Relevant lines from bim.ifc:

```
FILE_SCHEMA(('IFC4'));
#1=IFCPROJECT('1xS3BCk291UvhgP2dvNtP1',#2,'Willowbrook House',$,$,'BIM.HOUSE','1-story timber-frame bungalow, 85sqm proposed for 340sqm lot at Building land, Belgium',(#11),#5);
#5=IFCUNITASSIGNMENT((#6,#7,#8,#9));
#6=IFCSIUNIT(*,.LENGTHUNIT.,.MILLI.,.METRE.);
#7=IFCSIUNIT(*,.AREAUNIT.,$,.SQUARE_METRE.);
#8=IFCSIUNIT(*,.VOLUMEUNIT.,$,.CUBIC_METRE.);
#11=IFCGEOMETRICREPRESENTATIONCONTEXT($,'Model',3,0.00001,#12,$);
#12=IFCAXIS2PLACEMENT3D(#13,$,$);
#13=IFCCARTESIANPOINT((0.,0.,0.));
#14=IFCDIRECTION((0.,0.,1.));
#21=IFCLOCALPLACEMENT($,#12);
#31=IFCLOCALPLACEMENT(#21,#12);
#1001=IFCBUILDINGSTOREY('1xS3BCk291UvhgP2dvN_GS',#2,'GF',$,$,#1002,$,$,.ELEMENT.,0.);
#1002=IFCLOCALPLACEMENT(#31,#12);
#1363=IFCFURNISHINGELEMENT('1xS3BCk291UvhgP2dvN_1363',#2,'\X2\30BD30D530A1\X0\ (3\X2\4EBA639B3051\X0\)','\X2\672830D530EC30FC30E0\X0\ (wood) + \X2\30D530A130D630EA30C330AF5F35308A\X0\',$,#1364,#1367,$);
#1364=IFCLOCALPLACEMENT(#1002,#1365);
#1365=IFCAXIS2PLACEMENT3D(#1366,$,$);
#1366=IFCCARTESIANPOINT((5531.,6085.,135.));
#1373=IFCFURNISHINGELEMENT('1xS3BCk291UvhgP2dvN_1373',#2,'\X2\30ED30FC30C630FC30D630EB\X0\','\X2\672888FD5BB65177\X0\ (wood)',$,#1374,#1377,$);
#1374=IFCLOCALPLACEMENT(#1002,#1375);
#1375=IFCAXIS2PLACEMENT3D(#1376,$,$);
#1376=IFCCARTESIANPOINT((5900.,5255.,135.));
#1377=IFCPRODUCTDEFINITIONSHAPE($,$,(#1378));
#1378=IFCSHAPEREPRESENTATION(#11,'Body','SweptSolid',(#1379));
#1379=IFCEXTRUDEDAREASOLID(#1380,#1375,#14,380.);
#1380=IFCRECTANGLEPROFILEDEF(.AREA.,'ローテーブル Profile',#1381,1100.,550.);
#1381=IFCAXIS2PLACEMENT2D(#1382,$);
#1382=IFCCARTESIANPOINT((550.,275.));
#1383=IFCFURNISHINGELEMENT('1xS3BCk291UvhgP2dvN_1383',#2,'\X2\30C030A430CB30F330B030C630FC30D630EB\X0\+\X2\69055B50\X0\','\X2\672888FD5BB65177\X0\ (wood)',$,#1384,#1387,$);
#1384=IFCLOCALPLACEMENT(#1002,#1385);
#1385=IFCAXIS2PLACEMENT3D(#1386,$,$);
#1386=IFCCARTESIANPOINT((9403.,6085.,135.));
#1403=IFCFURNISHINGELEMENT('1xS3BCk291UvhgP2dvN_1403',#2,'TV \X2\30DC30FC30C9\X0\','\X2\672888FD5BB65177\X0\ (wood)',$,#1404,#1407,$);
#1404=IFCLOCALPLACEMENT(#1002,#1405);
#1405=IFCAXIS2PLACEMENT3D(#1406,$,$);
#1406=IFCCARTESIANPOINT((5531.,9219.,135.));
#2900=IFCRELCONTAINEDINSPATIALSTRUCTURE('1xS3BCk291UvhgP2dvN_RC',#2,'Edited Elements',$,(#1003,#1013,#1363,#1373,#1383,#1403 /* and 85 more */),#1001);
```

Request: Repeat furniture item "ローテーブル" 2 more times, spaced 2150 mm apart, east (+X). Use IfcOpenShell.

```python
import numpy as np
import ifcopenshell
import ifcopenshell.api.geometry
import ifcopenshell.api.root
import ifcopenshell.util.element
import ifcopenshell.util.placement
import ifcopenshell.util.unit

model = ifcopenshell.open("bim.ifc")
unit_scale = ifcopenshell.util.unit.calculate_unit_scale(model)


def reuse_history(source, copy):
    """copy_class also copies each property set's owner history, people and application; keep the originals."""
    for rel in copy.IsDefinedBy:
        if rel.is_a("IfcRelDefinesByProperties") and (history := rel.RelatingPropertyDefinition.OwnerHistory):
            rel.RelatingPropertyDefinition.OwnerHistory = source.OwnerHistory
            ifcopenshell.util.element.remove_deep2(model, history)


source = model.by_guid("1xS3BCk291UvhgP2dvN_1373")
base = ifcopenshell.util.placement.get_local_placement(source.ObjectPlacement)
step = np.array([1.0, 0.0, 0.0]) * 2.15 / unit_scale

for i in range(1, 3):
    copy = ifcopenshell.api.root.copy_class(model, product=source)
    copy.Representation = ifcopenshell.util.element.copy_deep(
        model, source.Representation, exclude=["IfcGeometricRepresentationContext", "IfcRepresentationMap"]
    )
    reuse_history(source, copy)
    matrix = base.copy()
    matrix[:3, 3] += i * step
    print("added at", matrix[:3, 3].round(3) + 0.0)
    ifcopenshell.api.geometry.edit_object_placement(model, product=copy, matrix=matrix, is_si=False)

model.write("bim_updated.ifc")
```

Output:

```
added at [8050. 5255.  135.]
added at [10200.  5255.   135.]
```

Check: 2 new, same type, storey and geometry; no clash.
